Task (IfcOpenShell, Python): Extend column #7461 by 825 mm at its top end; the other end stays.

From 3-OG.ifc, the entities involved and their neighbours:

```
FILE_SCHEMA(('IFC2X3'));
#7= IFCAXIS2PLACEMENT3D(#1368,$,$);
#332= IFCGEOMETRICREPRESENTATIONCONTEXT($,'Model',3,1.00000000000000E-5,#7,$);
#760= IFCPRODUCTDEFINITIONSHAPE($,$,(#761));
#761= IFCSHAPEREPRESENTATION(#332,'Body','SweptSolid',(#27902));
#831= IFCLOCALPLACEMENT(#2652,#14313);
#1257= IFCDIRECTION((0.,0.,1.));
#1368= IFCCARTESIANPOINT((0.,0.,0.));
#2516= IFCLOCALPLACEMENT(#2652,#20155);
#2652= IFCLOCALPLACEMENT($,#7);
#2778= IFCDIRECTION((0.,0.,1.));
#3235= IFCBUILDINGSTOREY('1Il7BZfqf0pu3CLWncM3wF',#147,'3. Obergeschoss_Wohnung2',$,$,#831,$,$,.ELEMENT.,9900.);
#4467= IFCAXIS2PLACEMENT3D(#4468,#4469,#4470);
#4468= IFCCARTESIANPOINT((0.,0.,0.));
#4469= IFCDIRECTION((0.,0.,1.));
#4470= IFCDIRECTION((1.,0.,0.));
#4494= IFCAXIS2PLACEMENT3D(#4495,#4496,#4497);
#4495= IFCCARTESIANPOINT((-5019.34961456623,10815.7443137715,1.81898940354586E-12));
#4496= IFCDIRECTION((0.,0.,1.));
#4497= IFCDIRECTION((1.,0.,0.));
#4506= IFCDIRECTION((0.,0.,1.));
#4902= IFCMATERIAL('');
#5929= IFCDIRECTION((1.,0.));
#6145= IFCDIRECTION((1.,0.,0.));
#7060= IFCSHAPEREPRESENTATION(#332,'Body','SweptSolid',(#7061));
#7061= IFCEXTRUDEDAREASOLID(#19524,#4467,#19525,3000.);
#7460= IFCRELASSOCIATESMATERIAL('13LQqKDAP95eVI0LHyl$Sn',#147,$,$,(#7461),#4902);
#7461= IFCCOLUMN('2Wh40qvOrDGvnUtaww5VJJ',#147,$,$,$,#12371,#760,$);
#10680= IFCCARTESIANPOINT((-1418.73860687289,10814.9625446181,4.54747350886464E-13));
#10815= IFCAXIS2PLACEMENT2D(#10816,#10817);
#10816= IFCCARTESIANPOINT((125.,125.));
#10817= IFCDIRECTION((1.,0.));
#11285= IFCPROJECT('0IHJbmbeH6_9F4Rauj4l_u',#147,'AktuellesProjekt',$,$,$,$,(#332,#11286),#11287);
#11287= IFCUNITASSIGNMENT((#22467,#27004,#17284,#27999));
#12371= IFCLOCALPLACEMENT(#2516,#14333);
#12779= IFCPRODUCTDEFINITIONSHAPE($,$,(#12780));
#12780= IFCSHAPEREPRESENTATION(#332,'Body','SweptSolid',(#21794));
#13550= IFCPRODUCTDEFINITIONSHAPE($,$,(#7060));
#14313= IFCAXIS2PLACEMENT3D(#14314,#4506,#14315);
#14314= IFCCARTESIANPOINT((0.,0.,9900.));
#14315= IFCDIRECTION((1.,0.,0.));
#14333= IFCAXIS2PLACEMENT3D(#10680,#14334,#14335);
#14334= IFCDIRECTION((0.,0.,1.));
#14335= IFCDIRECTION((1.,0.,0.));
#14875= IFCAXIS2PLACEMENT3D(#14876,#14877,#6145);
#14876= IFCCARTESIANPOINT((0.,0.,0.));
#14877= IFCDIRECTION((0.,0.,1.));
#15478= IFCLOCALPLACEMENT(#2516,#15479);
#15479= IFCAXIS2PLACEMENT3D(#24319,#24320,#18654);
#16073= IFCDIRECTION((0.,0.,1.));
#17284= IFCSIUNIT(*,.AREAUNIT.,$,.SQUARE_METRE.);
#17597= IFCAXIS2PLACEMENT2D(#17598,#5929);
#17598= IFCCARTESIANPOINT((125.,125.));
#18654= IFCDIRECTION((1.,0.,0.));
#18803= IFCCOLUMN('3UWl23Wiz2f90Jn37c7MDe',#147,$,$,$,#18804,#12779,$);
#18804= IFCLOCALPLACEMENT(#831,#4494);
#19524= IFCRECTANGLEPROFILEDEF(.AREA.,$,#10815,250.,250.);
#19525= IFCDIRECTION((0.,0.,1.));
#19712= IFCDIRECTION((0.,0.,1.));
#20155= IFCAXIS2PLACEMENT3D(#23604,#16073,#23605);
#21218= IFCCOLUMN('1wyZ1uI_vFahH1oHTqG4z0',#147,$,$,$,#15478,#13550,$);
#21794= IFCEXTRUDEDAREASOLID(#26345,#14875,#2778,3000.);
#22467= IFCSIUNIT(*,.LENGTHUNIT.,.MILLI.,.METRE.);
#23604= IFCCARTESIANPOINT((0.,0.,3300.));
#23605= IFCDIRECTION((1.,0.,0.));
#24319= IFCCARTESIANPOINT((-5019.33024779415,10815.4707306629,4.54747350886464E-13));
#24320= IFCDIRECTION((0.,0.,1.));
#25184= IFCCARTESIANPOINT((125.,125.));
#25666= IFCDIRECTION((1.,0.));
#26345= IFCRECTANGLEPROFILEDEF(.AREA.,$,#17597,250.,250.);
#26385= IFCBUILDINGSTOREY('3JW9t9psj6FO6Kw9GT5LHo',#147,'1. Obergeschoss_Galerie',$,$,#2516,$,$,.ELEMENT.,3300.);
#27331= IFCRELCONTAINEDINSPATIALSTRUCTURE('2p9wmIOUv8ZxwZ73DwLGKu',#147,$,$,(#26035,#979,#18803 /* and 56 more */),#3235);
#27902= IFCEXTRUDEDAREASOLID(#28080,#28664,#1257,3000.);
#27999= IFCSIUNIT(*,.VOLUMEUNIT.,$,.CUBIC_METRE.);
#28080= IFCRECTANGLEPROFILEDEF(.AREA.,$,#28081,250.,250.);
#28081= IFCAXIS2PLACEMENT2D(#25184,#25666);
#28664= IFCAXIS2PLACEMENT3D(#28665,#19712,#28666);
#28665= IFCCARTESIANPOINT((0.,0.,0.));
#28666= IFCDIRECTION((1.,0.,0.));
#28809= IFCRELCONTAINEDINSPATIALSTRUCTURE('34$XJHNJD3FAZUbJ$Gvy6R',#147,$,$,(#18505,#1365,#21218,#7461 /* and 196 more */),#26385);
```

```python
import ifcopenshell

model = ifcopenshell.open("3-OG.ifc")

member = model.by_id(7461)
change = 825.0

# The extrusion runs towards the end named, so only its depth changes.
body = next(r for r in member.Representation.Representations if r.RepresentationIdentifier == "Body")
solid = body.Items[0]
old_length = solid.Depth
solid.Depth += change

print(f"length {old_length:g} -> {solid.Depth:g}")

model.write("3-OG-out.ifc")
```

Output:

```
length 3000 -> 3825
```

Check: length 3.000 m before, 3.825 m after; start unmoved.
